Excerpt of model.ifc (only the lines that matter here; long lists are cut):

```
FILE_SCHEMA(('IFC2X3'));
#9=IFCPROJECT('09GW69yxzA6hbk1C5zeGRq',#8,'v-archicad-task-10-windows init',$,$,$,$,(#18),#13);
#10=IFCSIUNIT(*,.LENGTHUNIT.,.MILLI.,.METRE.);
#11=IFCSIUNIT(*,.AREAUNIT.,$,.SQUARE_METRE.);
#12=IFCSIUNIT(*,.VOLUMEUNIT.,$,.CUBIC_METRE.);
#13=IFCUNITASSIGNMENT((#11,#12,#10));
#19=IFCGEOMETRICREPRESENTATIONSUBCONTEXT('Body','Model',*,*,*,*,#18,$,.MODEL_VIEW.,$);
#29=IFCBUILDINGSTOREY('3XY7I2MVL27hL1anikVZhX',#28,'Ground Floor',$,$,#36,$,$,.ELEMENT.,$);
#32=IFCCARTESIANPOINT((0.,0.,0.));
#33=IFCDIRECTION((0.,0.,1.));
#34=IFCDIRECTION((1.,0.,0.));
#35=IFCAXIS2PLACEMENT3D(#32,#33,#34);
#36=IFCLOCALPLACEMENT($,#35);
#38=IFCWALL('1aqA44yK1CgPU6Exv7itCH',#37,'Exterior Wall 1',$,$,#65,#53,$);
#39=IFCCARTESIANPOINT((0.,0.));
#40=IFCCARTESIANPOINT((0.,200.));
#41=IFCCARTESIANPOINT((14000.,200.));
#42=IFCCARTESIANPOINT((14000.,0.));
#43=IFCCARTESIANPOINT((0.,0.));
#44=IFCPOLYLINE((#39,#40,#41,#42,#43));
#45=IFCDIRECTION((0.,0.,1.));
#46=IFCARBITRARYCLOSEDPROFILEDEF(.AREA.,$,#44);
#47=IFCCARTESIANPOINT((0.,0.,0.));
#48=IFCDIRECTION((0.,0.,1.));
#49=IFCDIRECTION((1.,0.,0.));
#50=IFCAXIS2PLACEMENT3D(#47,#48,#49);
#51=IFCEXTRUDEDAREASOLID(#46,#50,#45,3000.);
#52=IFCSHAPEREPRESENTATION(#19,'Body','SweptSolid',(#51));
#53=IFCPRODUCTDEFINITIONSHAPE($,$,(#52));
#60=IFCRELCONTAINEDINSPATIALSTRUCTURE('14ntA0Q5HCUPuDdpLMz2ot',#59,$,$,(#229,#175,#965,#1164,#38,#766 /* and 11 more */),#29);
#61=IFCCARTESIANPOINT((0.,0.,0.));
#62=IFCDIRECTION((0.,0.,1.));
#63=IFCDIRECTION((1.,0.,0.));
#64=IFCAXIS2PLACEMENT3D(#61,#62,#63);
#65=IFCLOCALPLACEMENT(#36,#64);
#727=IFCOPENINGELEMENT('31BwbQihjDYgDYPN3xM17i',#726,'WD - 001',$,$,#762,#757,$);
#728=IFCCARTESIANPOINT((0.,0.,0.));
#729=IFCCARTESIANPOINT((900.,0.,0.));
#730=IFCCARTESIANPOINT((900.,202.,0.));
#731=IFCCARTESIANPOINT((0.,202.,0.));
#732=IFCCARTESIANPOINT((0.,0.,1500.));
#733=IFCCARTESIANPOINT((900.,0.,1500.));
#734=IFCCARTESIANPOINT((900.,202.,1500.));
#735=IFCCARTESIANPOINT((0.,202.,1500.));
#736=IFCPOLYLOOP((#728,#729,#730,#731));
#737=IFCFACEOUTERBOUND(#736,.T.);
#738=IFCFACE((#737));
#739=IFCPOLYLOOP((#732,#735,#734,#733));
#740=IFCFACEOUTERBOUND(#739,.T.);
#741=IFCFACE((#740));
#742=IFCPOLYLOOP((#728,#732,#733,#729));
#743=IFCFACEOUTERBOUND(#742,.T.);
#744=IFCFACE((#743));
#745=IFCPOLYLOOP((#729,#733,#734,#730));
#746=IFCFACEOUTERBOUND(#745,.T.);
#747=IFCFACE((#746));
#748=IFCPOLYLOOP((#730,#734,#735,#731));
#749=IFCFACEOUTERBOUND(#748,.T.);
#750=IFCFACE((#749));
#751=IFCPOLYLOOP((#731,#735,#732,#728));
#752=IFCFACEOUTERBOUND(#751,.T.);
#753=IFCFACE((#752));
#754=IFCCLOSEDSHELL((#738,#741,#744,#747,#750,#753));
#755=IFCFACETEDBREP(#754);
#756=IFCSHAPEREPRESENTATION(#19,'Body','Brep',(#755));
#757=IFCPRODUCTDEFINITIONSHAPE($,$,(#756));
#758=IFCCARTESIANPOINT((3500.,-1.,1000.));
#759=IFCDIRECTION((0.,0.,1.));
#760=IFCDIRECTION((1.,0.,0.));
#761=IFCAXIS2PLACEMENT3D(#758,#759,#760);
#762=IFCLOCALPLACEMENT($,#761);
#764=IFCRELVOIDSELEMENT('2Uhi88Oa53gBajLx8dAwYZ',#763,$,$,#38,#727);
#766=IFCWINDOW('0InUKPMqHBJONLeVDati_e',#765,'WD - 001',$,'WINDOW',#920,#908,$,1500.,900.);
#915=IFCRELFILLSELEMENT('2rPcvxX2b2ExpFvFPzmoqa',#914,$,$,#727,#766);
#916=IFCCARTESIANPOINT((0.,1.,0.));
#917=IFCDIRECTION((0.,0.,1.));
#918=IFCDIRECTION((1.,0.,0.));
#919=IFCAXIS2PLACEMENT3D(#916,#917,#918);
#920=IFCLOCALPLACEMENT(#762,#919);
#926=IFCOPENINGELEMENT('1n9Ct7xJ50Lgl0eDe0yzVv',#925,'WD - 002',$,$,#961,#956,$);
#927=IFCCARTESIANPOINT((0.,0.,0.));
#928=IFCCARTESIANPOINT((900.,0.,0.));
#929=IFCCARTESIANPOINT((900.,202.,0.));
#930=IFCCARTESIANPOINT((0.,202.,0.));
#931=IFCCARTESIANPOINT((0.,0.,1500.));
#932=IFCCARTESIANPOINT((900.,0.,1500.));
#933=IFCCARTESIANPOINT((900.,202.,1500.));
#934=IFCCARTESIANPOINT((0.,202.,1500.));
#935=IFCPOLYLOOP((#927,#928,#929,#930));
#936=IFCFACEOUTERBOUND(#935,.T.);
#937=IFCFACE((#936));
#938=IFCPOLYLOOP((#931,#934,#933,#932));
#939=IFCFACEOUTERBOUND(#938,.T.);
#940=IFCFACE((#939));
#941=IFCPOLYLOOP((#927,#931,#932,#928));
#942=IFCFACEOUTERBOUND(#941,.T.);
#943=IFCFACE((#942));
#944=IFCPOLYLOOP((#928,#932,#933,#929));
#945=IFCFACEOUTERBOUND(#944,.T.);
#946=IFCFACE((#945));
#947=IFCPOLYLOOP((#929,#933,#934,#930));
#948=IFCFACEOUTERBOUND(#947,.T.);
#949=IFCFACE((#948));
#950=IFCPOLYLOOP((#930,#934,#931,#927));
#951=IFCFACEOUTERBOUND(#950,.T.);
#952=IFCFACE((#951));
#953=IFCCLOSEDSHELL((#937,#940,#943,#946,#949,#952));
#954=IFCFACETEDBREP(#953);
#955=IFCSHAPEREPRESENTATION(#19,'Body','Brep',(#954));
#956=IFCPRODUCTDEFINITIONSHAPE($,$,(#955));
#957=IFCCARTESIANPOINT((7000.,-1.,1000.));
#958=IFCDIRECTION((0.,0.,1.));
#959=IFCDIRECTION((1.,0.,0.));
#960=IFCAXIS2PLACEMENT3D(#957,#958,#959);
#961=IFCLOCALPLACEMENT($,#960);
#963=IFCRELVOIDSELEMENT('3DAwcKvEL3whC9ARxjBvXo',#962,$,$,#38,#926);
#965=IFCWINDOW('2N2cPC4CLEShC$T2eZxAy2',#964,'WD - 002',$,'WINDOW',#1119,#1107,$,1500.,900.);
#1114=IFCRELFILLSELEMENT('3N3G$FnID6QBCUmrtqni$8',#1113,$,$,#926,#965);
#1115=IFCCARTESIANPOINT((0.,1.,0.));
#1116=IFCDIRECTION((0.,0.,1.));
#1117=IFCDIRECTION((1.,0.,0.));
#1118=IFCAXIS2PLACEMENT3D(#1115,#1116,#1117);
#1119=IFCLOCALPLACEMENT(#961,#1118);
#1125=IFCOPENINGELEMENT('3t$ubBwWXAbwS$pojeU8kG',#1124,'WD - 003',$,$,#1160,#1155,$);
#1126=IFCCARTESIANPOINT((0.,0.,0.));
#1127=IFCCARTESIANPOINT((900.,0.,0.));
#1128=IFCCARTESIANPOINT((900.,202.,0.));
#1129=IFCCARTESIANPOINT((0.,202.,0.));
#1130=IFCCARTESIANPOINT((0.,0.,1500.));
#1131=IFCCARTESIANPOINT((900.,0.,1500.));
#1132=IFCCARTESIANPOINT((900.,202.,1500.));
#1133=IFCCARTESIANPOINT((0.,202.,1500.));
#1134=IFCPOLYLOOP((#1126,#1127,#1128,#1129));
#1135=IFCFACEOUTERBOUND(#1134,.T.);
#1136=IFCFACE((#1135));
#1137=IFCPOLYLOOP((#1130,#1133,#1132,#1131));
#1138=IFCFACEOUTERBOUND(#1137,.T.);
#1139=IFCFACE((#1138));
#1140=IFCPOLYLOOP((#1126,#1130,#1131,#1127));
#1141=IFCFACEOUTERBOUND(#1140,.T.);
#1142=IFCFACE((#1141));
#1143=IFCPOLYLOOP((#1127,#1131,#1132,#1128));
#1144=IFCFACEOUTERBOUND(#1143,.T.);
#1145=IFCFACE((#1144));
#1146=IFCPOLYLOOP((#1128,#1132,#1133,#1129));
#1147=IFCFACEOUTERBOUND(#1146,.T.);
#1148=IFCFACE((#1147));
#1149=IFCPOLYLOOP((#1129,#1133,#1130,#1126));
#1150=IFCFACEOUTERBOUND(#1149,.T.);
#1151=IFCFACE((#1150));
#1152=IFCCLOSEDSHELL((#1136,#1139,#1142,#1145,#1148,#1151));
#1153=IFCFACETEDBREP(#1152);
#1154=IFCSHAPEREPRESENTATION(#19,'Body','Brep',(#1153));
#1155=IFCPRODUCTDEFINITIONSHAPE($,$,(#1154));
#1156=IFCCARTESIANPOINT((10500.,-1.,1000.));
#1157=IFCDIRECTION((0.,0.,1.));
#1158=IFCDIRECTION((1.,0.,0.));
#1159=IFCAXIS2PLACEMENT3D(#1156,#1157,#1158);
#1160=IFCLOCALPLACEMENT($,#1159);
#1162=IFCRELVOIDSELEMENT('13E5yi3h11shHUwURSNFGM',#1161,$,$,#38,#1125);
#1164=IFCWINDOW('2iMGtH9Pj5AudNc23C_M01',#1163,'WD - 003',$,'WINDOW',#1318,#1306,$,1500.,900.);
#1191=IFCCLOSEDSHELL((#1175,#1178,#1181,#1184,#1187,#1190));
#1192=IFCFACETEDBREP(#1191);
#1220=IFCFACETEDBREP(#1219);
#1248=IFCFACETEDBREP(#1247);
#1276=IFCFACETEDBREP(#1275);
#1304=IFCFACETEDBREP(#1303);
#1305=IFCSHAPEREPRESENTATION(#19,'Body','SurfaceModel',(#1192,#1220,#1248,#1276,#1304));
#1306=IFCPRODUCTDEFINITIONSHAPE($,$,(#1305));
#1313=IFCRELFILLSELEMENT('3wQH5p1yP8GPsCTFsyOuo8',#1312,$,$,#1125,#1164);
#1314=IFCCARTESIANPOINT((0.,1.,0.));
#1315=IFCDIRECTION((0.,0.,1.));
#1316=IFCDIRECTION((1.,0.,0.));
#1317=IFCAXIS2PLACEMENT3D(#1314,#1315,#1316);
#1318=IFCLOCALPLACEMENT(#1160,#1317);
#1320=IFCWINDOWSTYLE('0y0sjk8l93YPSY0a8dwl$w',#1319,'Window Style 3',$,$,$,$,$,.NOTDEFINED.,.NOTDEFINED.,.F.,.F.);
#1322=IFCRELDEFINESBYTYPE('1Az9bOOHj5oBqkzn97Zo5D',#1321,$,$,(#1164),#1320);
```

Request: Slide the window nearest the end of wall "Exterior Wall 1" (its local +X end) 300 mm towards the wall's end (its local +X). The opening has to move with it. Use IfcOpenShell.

```python
import ifcopenshell
import ifcopenshell.api.geometry
import ifcopenshell.util.placement

model = ifcopenshell.open("model.ifc")

window = model.by_id(1164)
opening = window.FillsVoids[0].RelatingOpeningElement
wall = opening.VoidsElements[0].RelatingBuildingElement

wall_matrix = ifcopenshell.util.placement.get_local_placement(wall.ObjectPlacement)
shift = wall_matrix[:3, 0] * 300.0
before = ifcopenshell.util.placement.get_local_placement(window.ObjectPlacement)[:3, 3].copy()

# The window is placed relative to its opening, so it follows when the opening moves.
matrix = ifcopenshell.util.placement.get_local_placement(opening.ObjectPlacement)
matrix[:3, 3] += shift
ifcopenshell.api.geometry.edit_object_placement(
    model, product=opening, matrix=matrix, is_si=False, should_transform_children=True
)

after = ifcopenshell.util.placement.get_local_placement(window.ObjectPlacement)[:3, 3]
print("window moved by", (after - before).round(3) + 0.0)

model.write("model_rev.ifc")
```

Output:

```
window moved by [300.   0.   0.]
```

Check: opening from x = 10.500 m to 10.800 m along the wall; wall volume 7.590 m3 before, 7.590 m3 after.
